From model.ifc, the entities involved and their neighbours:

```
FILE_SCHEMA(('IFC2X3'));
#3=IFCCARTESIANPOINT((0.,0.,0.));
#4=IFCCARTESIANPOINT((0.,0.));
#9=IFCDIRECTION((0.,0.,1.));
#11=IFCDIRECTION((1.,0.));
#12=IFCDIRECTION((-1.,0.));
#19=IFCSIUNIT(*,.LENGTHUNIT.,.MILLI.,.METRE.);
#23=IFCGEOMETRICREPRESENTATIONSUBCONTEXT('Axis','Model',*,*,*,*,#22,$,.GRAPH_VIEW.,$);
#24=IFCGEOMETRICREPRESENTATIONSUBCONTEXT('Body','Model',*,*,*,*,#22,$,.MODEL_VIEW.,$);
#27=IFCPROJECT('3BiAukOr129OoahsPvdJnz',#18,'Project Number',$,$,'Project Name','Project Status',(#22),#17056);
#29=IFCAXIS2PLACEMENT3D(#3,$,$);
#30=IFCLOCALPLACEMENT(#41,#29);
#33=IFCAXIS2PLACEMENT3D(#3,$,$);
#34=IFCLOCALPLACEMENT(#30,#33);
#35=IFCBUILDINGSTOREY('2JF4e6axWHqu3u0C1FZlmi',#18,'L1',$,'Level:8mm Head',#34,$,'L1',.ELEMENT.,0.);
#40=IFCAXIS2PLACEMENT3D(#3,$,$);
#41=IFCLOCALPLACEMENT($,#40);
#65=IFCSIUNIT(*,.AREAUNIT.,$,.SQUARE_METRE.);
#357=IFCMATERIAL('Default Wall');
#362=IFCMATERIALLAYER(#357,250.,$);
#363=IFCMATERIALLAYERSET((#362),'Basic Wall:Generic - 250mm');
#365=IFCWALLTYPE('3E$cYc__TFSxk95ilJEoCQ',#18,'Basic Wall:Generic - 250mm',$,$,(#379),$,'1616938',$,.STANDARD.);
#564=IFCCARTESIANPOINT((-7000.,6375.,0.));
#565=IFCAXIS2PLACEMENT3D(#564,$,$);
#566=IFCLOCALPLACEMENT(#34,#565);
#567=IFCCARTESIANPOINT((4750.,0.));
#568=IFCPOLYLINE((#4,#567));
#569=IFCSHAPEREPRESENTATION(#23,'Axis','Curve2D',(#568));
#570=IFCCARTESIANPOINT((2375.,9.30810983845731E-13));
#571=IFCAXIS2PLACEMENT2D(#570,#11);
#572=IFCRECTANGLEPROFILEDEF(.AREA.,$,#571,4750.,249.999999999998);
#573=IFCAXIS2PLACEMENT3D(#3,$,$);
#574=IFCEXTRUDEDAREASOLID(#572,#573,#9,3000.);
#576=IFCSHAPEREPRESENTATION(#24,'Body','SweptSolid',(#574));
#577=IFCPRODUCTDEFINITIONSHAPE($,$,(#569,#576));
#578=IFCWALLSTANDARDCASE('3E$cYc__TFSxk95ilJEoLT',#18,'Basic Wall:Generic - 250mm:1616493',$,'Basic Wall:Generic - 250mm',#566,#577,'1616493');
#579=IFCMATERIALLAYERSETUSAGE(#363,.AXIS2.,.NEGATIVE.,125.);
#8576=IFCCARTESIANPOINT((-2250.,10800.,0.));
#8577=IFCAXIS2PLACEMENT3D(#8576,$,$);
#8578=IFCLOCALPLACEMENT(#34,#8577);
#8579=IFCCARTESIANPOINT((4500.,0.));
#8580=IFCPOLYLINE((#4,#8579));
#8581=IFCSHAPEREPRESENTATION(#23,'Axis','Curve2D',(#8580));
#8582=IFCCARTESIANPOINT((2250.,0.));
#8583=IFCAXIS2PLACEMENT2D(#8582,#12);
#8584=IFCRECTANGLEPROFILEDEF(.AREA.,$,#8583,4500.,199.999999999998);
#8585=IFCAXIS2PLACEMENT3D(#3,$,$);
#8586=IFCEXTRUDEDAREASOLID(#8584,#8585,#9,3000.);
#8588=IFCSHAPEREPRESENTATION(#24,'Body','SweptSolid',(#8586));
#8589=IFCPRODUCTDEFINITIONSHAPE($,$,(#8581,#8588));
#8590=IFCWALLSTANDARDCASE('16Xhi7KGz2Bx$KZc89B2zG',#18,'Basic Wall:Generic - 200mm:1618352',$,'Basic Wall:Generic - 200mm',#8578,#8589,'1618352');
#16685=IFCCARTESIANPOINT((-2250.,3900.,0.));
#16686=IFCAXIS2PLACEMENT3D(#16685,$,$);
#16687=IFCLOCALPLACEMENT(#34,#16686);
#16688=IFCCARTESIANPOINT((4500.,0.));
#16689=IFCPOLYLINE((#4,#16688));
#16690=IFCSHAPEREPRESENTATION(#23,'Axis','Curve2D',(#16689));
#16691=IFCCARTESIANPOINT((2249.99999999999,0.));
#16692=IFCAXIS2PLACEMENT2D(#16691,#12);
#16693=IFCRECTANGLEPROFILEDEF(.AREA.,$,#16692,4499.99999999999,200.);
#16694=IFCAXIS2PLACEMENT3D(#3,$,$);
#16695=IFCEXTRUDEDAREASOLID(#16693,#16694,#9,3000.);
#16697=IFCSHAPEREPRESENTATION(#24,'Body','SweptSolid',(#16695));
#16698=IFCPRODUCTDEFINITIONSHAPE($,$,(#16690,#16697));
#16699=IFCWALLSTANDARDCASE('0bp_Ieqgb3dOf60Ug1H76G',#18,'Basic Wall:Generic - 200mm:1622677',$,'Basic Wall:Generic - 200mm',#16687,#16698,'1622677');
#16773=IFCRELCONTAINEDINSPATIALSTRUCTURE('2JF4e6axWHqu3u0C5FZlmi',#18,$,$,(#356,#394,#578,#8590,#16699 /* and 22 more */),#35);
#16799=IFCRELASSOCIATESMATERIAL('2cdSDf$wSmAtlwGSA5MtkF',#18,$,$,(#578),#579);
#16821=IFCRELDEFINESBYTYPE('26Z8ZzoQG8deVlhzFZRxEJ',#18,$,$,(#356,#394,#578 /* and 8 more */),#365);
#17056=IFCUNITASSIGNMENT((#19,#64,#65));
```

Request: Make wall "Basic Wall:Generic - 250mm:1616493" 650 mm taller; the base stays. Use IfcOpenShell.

```python
import ifcopenshell
import ifcopenshell.geom
import ifcopenshell.util.representation
import ifcopenshell.util.shape
import ifcopenshell.util.unit

model = ifcopenshell.open("model.ifc")
unit_scale = ifcopenshell.util.unit.calculate_unit_scale(model)
settings = ifcopenshell.geom.settings()


def volume(element):
    """Net volume in cubic metres, openings subtracted."""
    shape = ifcopenshell.geom.create_shape(settings, element)
    return ifcopenshell.util.shape.get_volume(shape.geometry)


wall = model.by_id(578)
before = volume(wall)

body = ifcopenshell.util.representation.get_representation(wall, "Model", "Body")
solid = body.Items[0]
old_height = solid.Depth
solid.Depth += 0.65 / unit_scale
after = volume(wall)

print(f"height {old_height:g} -> {solid.Depth:g}, volume {before:.3f} -> {after:.3f} m3")

model.write("model-out.ifc")
```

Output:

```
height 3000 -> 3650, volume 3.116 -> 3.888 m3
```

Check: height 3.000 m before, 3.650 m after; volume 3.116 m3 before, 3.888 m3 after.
